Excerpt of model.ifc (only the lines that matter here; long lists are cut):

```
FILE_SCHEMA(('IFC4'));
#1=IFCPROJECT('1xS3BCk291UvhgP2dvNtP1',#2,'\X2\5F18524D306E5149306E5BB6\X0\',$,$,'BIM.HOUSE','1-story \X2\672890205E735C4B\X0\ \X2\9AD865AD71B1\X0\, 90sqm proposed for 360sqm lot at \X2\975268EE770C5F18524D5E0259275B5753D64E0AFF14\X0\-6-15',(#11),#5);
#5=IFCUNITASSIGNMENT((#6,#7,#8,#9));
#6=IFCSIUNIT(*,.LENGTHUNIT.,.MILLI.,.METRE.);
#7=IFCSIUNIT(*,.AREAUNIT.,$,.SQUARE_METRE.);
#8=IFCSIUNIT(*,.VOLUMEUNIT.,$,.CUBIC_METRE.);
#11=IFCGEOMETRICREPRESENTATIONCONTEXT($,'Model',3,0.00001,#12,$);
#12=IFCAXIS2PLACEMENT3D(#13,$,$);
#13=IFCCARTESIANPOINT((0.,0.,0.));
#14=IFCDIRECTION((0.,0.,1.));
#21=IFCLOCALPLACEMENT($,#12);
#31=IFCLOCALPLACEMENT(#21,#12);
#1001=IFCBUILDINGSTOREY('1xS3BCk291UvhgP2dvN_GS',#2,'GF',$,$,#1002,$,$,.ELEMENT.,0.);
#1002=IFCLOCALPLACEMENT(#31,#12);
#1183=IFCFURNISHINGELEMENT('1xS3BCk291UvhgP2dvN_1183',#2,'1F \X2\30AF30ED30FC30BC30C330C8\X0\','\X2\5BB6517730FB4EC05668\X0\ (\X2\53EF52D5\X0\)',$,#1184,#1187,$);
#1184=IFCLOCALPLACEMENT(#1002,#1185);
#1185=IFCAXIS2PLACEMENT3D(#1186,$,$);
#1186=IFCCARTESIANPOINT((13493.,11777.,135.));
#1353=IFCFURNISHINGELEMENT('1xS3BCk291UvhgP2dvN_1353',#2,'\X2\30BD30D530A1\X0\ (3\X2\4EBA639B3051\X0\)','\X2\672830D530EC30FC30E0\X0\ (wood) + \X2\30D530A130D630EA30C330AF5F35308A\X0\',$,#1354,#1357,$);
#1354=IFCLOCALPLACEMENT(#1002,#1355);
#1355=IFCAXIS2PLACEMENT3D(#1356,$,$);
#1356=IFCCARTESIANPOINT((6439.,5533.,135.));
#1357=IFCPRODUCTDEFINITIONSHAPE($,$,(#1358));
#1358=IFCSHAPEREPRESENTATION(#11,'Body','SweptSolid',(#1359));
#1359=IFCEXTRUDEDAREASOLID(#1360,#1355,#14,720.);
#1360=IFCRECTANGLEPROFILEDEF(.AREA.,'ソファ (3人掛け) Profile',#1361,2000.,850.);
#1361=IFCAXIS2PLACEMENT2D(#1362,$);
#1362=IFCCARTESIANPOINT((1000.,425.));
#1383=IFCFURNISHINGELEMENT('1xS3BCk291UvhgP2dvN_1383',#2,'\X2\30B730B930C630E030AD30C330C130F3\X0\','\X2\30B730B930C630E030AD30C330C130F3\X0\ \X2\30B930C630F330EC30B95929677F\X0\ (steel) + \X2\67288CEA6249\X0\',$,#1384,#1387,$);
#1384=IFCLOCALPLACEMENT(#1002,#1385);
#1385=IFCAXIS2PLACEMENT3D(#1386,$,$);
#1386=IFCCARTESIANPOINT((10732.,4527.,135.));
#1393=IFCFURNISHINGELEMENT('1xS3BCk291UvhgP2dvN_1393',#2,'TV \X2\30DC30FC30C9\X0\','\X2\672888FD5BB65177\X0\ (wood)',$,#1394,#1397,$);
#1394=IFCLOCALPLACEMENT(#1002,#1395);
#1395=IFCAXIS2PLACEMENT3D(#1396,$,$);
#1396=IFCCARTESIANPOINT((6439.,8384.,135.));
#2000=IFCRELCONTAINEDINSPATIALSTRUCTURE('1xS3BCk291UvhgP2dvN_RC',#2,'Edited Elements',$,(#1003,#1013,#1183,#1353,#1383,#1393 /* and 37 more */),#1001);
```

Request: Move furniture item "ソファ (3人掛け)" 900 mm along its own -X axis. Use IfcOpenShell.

```python
import ifcopenshell
import ifcopenshell.api.geometry
import ifcopenshell.util.placement
import ifcopenshell.util.unit

model = ifcopenshell.open("model.ifc")
unit_scale = ifcopenshell.util.unit.calculate_unit_scale(model)

item = model.by_guid("1xS3BCk291UvhgP2dvN_1353")
matrix = ifcopenshell.util.placement.get_local_placement(item.ObjectPlacement)
matrix[:3, 3] -= matrix[:3, 0] * 0.9 / unit_scale
ifcopenshell.api.geometry.edit_object_placement(model, product=item, matrix=matrix, is_si=False)

print(ifcopenshell.util.placement.get_local_placement(item.ObjectPlacement).round(3) + 0.0)

model.write("model_edited.ifc")
```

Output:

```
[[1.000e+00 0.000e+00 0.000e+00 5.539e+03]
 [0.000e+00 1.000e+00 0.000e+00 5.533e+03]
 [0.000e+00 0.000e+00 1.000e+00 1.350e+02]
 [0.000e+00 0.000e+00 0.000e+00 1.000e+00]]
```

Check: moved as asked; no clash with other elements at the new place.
